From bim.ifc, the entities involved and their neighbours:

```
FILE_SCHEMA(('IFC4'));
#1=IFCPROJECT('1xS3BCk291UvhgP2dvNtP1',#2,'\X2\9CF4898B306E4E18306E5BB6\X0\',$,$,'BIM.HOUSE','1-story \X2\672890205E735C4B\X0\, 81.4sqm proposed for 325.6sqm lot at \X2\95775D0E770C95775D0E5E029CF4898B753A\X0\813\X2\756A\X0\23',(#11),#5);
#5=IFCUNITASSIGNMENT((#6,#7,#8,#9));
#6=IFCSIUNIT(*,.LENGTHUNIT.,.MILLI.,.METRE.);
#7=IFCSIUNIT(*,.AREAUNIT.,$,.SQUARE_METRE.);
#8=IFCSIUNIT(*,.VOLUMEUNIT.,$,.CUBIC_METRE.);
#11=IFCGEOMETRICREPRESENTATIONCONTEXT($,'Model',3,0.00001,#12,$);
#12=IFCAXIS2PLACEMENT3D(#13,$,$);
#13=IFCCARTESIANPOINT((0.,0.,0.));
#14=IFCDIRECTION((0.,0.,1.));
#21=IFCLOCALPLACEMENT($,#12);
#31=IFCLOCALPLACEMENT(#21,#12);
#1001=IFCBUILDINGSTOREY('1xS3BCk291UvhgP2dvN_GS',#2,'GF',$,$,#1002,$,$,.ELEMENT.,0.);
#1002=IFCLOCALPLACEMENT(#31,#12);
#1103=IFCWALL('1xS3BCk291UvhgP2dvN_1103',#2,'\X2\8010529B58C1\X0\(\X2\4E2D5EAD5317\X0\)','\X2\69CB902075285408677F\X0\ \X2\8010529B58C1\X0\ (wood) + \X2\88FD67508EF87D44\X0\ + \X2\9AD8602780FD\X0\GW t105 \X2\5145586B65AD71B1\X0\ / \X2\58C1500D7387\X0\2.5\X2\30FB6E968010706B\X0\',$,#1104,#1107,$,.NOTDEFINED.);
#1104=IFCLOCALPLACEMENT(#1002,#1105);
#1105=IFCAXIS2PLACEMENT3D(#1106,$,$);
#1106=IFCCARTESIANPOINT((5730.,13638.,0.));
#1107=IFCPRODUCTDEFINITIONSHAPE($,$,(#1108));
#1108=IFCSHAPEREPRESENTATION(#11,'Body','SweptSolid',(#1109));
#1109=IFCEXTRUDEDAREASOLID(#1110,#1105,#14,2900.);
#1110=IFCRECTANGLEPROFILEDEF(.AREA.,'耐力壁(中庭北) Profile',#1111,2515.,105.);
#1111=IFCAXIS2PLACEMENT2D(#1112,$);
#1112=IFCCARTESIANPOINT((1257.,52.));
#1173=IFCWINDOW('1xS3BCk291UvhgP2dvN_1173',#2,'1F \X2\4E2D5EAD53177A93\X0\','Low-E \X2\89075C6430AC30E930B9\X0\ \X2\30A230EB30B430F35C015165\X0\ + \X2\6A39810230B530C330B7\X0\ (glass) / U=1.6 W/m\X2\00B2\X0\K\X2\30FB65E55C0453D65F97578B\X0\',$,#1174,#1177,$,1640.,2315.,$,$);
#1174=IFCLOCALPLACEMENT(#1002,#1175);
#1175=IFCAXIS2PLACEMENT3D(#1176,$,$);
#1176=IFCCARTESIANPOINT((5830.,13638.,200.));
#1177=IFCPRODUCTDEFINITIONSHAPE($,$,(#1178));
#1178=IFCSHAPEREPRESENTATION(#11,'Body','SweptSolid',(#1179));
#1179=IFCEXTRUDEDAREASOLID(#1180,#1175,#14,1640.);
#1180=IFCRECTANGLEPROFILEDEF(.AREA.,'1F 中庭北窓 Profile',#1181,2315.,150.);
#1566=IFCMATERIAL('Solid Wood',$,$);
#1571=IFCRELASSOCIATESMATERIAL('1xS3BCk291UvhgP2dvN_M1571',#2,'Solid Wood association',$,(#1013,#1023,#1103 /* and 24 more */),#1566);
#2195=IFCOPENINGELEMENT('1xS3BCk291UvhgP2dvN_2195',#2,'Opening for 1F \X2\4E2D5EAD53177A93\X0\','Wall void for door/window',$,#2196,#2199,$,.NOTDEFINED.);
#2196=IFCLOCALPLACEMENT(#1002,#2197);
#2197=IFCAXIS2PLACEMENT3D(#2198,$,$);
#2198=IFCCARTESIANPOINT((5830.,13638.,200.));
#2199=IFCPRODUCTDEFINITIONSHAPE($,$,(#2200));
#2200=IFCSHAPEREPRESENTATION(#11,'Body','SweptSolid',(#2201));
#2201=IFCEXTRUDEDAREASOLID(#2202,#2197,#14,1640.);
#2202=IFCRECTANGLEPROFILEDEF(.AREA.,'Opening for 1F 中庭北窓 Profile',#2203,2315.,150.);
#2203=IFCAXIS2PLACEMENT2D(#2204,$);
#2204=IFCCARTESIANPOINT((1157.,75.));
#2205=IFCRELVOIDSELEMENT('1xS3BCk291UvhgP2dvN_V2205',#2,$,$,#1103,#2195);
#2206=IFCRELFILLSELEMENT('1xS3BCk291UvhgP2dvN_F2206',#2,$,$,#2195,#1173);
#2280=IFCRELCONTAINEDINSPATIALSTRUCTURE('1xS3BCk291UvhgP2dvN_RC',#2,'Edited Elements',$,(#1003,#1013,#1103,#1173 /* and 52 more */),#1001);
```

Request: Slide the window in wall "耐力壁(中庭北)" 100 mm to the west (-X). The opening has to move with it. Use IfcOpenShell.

```python
import ifcopenshell
import ifcopenshell.api.geometry
import ifcopenshell.util.placement

model = ifcopenshell.open("bim.ifc")

window = model.by_guid("1xS3BCk291UvhgP2dvN_1173")
opening = window.FillsVoids[0].RelatingOpeningElement
wall = opening.VoidsElements[0].RelatingBuildingElement

wall_matrix = ifcopenshell.util.placement.get_local_placement(wall.ObjectPlacement)
shift = wall_matrix[:3, 0] * -100.0
before = ifcopenshell.util.placement.get_local_placement(window.ObjectPlacement)[:3, 3].copy()

# The window is not placed relative to its opening, so move both.
for product in (opening, window):
    matrix = ifcopenshell.util.placement.get_local_placement(product.ObjectPlacement)
    matrix[:3, 3] += shift
    ifcopenshell.api.geometry.edit_object_placement(model, product=product, matrix=matrix, is_si=False)

after = ifcopenshell.util.placement.get_local_placement(window.ObjectPlacement)[:3, 3]
print("window moved by", (after - before).round(3) + 0.0)

model.write("bim_edited.ifc")
```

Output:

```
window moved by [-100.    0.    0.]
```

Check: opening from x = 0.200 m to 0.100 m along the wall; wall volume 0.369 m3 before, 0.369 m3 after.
